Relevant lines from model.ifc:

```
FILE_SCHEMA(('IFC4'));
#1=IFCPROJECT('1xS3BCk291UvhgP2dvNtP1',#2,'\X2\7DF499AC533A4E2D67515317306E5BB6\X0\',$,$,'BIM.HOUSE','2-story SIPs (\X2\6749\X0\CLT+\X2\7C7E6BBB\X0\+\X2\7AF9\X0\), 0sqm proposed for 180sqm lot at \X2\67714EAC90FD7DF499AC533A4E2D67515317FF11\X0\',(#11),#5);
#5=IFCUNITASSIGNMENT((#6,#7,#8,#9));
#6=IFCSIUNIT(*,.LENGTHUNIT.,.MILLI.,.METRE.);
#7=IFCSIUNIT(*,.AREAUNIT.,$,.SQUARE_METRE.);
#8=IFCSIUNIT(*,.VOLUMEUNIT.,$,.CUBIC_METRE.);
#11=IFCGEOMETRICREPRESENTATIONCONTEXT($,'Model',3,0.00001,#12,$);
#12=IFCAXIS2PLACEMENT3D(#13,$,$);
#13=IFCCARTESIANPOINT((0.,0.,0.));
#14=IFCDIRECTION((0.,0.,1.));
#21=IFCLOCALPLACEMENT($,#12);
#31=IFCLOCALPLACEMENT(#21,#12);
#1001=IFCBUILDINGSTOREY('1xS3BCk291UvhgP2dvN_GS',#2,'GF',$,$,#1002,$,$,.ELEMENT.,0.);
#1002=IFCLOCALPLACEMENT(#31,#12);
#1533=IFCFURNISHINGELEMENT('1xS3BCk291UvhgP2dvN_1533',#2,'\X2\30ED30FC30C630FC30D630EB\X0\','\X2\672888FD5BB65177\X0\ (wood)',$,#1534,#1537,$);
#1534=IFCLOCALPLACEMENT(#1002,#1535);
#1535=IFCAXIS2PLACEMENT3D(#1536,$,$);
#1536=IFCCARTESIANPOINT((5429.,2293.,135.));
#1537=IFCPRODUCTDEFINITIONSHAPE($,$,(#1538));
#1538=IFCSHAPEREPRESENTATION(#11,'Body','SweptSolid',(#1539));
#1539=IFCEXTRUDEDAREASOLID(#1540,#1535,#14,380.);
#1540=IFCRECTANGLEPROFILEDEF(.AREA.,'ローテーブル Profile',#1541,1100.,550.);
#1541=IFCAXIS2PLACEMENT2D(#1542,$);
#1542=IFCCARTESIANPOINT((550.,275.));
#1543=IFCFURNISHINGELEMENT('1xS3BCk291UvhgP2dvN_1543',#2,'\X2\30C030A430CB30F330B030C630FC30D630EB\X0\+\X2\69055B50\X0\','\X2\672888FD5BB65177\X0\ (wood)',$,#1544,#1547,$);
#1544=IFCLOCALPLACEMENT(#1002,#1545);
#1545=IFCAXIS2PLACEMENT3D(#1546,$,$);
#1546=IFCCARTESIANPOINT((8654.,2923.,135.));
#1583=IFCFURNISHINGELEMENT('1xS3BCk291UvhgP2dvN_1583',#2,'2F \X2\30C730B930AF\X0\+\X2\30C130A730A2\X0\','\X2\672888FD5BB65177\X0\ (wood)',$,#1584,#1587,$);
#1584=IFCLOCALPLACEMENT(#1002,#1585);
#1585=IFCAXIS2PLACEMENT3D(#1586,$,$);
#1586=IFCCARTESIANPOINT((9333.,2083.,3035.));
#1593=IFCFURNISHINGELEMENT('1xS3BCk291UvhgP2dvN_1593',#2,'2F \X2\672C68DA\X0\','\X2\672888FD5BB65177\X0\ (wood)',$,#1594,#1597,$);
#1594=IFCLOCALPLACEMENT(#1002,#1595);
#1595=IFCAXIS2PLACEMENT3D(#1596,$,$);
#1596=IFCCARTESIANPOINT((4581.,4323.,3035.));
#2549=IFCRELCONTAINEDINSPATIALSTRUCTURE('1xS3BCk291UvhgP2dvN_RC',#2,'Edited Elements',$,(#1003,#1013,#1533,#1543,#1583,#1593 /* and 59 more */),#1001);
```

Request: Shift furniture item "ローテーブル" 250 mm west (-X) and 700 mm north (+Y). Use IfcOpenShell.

```python
import ifcopenshell
import ifcopenshell.api.geometry
import ifcopenshell.util.placement

model = ifcopenshell.open("model.ifc")

item = model.by_guid("1xS3BCk291UvhgP2dvN_1533")
matrix = ifcopenshell.util.placement.get_local_placement(item.ObjectPlacement)
matrix[0, 3] -= 250.0
matrix[1, 3] += 700.0
ifcopenshell.api.geometry.edit_object_placement(model, product=item, matrix=matrix, is_si=False)

print(ifcopenshell.util.placement.get_local_placement(item.ObjectPlacement).round(3) + 0.0)

model.write("model-out.ifc")
```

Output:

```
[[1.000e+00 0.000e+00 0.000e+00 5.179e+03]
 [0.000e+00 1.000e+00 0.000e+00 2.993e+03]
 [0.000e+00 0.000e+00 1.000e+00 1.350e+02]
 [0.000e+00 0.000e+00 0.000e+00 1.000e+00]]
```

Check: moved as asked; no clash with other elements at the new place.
